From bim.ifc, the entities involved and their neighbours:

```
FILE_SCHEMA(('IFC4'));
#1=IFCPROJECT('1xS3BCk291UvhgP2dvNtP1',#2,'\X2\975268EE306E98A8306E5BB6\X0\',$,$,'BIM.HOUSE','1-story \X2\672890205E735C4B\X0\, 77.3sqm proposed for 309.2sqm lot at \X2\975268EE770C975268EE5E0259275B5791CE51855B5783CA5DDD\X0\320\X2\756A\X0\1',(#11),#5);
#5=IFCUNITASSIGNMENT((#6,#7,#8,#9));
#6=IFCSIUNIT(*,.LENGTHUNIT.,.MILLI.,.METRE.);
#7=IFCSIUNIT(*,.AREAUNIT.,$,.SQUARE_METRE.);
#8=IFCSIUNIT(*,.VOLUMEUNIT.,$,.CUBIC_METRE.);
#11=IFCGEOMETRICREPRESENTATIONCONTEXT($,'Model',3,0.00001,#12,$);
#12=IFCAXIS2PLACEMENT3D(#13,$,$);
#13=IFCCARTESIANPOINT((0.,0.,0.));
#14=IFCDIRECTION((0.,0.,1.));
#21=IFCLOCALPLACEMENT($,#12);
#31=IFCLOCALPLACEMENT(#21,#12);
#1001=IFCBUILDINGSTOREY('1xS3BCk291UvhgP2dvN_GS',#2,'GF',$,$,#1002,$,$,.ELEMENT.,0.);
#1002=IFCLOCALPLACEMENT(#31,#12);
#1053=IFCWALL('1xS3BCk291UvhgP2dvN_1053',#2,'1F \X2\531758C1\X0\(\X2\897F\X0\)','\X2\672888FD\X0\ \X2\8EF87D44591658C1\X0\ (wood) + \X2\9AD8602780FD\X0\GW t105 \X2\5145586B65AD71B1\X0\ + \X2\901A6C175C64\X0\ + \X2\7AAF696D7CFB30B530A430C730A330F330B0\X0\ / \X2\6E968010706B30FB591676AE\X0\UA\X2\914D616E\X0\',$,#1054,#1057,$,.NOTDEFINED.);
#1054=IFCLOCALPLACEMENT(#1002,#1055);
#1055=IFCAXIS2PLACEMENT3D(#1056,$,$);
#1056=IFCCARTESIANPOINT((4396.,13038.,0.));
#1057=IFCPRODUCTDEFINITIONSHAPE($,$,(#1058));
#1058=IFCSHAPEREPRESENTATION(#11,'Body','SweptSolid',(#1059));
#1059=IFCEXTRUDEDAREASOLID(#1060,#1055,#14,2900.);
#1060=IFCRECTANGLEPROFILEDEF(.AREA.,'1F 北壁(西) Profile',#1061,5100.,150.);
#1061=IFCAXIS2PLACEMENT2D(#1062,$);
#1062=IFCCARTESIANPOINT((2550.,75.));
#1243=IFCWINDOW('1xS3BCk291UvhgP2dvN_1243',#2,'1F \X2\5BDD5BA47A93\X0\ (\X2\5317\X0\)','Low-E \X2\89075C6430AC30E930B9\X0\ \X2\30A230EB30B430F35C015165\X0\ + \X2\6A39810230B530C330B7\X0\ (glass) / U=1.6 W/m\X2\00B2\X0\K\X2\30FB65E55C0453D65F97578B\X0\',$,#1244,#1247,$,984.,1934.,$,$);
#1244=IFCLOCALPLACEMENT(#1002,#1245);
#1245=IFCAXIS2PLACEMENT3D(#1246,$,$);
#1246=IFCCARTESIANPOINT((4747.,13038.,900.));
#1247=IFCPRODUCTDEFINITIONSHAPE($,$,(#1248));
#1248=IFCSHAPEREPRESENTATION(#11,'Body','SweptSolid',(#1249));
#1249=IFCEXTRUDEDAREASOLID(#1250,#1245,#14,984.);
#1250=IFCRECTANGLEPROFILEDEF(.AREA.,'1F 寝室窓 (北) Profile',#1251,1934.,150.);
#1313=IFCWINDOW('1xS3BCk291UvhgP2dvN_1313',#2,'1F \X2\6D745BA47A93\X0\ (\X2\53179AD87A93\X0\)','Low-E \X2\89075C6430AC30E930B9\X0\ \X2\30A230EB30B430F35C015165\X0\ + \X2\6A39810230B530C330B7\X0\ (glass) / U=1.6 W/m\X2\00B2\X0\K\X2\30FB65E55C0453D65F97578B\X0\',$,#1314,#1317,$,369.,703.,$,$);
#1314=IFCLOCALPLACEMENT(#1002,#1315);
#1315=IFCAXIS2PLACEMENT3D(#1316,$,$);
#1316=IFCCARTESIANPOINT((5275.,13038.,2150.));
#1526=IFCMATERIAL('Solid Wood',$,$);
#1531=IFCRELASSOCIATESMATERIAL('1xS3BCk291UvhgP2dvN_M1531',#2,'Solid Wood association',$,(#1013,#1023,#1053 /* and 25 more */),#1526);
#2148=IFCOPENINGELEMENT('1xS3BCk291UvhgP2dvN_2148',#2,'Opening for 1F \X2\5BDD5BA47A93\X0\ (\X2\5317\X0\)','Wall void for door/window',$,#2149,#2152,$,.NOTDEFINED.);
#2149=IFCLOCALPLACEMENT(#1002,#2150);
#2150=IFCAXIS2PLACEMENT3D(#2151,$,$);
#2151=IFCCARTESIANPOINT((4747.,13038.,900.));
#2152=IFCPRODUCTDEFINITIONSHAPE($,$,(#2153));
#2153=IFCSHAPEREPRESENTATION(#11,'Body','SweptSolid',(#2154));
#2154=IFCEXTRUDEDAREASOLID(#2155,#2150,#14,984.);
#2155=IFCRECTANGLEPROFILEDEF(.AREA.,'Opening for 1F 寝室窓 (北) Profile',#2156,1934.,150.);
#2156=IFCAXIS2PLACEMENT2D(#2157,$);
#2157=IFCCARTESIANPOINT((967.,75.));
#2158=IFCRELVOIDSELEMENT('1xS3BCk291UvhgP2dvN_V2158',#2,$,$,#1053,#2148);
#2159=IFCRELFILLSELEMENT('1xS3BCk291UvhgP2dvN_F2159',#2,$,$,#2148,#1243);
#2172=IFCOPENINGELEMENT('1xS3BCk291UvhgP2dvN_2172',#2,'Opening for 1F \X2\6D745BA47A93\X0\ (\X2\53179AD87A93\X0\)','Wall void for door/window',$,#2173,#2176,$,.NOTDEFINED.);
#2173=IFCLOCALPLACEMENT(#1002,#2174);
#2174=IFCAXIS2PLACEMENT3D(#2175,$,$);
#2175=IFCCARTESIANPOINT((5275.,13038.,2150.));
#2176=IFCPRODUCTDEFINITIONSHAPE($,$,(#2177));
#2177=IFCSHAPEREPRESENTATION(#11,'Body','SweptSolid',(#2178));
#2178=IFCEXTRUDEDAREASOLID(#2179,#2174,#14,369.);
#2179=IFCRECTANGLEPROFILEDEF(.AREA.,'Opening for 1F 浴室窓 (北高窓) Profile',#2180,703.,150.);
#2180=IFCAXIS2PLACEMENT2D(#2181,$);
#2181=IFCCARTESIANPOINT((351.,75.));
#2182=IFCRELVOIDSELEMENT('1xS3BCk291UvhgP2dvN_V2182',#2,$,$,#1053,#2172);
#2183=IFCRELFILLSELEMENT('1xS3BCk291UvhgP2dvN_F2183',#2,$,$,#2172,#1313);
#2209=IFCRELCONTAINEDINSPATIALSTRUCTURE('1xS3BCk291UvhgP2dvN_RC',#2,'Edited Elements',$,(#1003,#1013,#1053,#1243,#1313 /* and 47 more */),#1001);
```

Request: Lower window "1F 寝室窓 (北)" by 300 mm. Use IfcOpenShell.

```python
import numpy as np
import ifcopenshell
import ifcopenshell.api.geometry
import ifcopenshell.util.placement
import ifcopenshell.util.unit

model = ifcopenshell.open("bim.ifc")
unit_scale = ifcopenshell.util.unit.calculate_unit_scale(model)

window = model.by_guid("1xS3BCk291UvhgP2dvN_1243")
opening = window.FillsVoids[0].RelatingOpeningElement
dz = -0.3 / unit_scale

shift = np.array([0.0, 0.0, dz])
# The window is not placed relative to its opening, so move both.
for product in (opening, window):
    matrix = ifcopenshell.util.placement.get_local_placement(product.ObjectPlacement)
    matrix[:3, 3] += shift
    ifcopenshell.api.geometry.edit_object_placement(model, product=product, matrix=matrix, is_si=False)

print(f"moved by {dz * unit_scale:+.3f} m")

model.write("bim_v2.ifc")
```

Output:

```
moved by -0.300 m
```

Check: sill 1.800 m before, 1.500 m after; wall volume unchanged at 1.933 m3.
